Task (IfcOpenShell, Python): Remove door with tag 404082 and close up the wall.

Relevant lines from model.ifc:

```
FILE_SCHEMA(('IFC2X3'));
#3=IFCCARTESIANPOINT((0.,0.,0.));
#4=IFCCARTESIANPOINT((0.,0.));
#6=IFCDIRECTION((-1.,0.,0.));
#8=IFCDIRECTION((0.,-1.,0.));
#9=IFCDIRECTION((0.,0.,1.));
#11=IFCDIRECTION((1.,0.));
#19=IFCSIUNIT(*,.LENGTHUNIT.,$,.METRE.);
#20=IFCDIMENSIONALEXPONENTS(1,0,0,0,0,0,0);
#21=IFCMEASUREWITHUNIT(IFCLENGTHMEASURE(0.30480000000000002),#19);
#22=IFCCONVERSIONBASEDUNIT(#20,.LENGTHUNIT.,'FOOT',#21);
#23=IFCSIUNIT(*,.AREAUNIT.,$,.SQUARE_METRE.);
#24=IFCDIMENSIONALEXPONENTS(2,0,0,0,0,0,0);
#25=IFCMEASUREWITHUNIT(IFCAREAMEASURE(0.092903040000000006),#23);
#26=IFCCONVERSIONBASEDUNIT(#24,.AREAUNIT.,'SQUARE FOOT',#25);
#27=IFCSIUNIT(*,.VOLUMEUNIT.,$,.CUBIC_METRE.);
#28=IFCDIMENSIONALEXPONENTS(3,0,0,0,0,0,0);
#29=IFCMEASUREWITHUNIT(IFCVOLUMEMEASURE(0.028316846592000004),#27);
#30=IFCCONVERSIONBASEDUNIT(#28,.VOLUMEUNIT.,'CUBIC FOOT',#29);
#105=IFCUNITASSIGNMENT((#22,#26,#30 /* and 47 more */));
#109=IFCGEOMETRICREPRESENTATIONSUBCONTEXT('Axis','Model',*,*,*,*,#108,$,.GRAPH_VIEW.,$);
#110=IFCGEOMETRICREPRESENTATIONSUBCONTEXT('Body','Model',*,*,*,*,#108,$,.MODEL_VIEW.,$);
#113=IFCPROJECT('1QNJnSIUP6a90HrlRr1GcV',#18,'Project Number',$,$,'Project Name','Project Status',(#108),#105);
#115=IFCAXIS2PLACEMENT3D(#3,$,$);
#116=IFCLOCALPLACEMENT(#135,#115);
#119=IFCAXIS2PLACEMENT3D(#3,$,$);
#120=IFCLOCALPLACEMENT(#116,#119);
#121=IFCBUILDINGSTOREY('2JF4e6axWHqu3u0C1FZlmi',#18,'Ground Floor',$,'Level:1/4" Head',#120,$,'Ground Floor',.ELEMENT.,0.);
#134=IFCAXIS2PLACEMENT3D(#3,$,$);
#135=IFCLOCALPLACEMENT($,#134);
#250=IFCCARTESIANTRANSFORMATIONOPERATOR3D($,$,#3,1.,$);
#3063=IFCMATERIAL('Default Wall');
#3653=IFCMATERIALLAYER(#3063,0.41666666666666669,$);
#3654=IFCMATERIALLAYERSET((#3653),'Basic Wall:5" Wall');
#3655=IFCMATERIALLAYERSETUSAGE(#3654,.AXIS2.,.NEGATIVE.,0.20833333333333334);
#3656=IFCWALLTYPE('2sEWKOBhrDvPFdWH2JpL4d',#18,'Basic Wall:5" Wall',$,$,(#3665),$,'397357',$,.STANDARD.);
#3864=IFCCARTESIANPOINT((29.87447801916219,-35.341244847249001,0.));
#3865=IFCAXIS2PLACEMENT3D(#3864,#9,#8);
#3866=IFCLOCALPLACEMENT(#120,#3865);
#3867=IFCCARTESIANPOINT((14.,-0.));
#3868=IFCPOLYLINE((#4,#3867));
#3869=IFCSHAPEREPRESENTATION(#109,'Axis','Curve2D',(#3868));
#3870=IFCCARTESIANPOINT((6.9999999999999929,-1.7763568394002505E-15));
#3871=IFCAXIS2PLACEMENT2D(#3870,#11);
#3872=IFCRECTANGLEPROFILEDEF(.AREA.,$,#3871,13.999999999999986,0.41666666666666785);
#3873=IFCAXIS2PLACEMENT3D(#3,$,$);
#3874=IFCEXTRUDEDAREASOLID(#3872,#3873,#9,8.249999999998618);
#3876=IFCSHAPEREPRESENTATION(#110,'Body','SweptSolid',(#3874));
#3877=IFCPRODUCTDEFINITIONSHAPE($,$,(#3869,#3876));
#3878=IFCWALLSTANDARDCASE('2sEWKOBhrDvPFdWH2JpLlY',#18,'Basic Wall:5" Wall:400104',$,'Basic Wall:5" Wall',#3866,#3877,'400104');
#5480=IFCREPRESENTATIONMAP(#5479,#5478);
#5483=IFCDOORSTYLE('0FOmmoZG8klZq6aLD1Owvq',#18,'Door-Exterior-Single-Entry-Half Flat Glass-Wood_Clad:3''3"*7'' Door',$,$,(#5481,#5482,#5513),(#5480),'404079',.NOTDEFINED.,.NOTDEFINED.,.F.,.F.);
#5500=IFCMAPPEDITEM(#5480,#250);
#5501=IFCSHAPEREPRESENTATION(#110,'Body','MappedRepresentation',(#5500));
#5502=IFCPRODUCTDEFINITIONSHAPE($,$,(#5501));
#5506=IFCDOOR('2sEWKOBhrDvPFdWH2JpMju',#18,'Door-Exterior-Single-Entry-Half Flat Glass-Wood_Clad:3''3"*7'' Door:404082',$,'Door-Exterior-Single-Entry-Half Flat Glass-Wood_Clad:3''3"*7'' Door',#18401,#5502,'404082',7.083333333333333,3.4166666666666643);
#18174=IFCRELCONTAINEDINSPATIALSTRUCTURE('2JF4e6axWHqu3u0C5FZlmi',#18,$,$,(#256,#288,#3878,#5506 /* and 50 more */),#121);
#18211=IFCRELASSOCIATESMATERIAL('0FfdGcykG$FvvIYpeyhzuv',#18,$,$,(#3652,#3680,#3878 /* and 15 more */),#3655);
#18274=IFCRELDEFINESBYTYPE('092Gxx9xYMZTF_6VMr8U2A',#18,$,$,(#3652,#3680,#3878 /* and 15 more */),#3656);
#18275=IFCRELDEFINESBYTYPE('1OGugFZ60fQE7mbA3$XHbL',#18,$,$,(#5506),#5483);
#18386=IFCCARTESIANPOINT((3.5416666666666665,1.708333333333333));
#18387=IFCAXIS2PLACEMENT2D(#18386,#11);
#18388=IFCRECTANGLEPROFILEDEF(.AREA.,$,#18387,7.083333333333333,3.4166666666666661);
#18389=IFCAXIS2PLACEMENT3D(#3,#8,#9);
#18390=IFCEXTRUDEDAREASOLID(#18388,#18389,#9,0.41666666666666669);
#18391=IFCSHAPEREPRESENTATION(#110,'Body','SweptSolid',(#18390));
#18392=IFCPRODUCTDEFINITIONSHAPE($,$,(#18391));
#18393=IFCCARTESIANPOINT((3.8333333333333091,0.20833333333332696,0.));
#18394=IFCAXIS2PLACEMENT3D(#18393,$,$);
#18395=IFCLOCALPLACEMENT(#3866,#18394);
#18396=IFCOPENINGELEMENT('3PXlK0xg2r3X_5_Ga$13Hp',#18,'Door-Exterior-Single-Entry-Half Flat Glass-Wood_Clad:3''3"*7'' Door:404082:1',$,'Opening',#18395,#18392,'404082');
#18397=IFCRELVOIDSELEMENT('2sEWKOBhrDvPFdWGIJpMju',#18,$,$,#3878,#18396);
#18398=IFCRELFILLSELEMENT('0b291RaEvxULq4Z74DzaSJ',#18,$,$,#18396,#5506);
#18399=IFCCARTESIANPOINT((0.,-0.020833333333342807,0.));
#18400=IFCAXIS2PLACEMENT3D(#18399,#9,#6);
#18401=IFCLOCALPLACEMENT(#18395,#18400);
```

```python
import ifcopenshell
import ifcopenshell.api.feature
import ifcopenshell.api.root
import ifcopenshell.geom
import ifcopenshell.util.shape

model = ifcopenshell.open("model.ifc")
settings = ifcopenshell.geom.settings()


def volume(element):
    """Net volume in cubic metres, openings subtracted."""
    shape = ifcopenshell.geom.create_shape(settings, element)
    return ifcopenshell.util.shape.get_volume(shape.geometry)


door = model.by_guid("2sEWKOBhrDvPFdWH2JpMju")
opening = door.FillsVoids[0].RelatingOpeningElement
wall = opening.VoidsElements[0].RelatingBuildingElement
before = volume(wall)

ifcopenshell.api.root.remove_product(model, product=door)
ifcopenshell.api.feature.remove_feature(model, feature=opening)

after = volume(wall)

print(f"wall volume {before:.3f} -> {after:.3f} m3")

model.write("model_v2.ifc")
```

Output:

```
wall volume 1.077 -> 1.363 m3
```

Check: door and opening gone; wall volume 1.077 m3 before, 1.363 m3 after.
